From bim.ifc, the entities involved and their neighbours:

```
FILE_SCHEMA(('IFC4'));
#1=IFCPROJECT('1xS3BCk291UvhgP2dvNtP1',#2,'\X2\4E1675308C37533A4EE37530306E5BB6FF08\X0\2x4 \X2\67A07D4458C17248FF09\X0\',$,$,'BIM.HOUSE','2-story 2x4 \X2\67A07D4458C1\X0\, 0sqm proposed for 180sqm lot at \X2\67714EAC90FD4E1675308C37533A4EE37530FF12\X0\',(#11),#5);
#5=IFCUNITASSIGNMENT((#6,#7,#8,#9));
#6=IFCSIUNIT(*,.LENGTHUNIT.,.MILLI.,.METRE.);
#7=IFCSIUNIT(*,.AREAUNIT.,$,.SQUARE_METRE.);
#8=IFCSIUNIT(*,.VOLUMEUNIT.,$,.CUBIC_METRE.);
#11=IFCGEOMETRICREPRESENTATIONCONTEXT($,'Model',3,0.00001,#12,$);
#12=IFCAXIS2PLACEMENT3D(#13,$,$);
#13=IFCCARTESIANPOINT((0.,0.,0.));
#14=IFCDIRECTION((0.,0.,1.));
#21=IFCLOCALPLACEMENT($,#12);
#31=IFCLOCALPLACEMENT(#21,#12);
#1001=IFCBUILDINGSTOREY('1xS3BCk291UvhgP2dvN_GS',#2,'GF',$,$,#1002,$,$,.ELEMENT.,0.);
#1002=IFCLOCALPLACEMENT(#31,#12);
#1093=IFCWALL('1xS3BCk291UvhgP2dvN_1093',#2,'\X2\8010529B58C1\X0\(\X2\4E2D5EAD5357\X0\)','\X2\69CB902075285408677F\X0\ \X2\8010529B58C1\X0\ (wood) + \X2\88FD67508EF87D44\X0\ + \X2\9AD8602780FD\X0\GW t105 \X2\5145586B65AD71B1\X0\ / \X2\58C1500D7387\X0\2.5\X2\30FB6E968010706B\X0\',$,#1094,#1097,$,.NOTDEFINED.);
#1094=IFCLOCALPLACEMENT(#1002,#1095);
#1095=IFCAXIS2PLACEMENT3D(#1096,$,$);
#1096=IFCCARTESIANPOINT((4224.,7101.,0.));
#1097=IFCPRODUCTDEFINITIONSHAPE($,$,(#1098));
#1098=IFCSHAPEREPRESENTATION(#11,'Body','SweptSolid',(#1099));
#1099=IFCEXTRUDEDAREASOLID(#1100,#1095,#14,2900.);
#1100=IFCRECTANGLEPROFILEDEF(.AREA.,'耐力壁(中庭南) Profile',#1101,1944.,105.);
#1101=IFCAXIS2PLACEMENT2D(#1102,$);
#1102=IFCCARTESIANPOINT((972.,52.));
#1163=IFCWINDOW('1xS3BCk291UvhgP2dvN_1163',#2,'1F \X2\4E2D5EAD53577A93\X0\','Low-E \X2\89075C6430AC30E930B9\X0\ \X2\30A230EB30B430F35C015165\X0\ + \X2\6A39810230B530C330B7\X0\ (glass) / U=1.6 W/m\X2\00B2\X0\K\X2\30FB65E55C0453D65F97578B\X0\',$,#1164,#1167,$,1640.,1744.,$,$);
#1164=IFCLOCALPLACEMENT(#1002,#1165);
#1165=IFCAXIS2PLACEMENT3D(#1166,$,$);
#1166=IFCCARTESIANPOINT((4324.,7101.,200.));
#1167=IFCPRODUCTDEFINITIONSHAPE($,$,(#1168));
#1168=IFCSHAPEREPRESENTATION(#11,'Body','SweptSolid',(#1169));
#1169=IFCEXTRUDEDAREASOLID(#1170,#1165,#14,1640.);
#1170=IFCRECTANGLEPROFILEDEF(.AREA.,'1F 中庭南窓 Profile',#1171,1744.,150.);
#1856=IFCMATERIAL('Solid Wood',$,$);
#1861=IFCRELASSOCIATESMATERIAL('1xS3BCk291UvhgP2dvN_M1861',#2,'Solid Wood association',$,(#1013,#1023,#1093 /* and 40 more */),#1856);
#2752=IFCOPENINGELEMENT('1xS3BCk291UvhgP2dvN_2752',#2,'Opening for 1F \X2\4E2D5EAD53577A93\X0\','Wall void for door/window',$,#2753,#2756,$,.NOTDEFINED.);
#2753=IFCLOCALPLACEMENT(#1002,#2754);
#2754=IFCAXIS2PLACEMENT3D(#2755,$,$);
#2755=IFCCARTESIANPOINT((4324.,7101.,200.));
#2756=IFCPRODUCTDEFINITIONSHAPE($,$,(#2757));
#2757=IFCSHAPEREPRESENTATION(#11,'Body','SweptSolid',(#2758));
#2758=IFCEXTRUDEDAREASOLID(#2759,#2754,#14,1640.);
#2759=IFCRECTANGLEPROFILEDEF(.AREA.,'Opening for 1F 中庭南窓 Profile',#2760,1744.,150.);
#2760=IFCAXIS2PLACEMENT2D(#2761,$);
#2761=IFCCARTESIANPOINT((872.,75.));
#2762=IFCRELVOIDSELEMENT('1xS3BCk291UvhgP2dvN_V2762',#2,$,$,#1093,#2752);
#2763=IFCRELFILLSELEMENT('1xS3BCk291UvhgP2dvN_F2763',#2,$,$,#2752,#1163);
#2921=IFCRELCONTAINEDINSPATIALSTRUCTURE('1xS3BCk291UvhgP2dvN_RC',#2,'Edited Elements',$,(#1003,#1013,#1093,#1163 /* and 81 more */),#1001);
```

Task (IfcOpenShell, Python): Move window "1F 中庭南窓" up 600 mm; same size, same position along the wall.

```python
import numpy as np
import ifcopenshell
import ifcopenshell.api.geometry
import ifcopenshell.util.placement
import ifcopenshell.util.unit

model = ifcopenshell.open("bim.ifc")
unit_scale = ifcopenshell.util.unit.calculate_unit_scale(model)

window = model.by_id(1163)
opening = window.FillsVoids[0].RelatingOpeningElement
dz = 600.0

shift = np.array([0.0, 0.0, dz])
# The window is not placed relative to its opening, so move both.
for product in (opening, window):
    matrix = ifcopenshell.util.placement.get_local_placement(product.ObjectPlacement)
    matrix[:3, 3] += shift
    ifcopenshell.api.geometry.edit_object_placement(model, product=product, matrix=matrix, is_si=False)

print(f"moved by {dz * unit_scale:+.3f} m")

model.write("bim_v2.ifc")
```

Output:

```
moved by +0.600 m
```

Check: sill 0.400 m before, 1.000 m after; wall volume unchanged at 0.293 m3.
